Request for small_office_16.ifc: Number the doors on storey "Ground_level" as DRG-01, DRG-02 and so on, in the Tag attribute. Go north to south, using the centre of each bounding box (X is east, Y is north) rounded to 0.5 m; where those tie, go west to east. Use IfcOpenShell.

First a look at what the model holds.

```python
import ifcopenshell
import ifcopenshell.util.element
import ifcopenshell.util.placement

model = ifcopenshell.open("small_office_16.ifc")
print(model.schema)
storey = next(s for s in model.by_type("IfcBuildingStorey") if s.Name == "Ground_level")
doors = [e for e in ifcopenshell.util.element.get_decomposition(storey) if e.is_a("IfcDoor")]
for e in sorted(doors, key=lambda e: e.id()):
    origin = ifcopenshell.util.placement.get_local_placement(e.ObjectPlacement)[:3, 3]
    print(e.id(), e.Tag, e.Name, origin.round(2) + 0.0, sep=" | ")
```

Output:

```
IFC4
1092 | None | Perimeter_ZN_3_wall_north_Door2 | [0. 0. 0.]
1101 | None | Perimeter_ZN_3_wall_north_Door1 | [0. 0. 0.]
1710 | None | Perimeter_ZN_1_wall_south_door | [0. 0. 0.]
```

```python
import ifcopenshell
import ifcopenshell.geom
import ifcopenshell.util.element
import ifcopenshell.util.shape

model = ifcopenshell.open("small_office_16.ifc")
settings = ifcopenshell.geom.settings()
settings.set("use-world-coords", True)


def centre(element):
    shape = ifcopenshell.geom.create_shape(settings, element)
    return ifcopenshell.util.shape.get_bbox_centroid(shape.geometry)


storey = next(s for s in model.by_type("IfcBuildingStorey") if s.Name == "Ground_level")
doors = [e for e in ifcopenshell.util.element.get_decomposition(storey) if e.is_a("IfcDoor")]

# Insertion points can sit at a corner or the storey origin, so sort by the geometry (in metres).
centres = {e: centre(e) for e in doors}
doors.sort(key=lambda e: (-round(centres[e][1] / 0.5), centres[e][0]))

for i, e in enumerate(doors, start=1):
    number = f"DRG-{i:02d}"
    e.Tag = number
    print(e.id(), number)

model.write("small_office_16_updated.ifc")
```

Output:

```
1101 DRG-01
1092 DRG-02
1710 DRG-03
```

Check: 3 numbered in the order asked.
